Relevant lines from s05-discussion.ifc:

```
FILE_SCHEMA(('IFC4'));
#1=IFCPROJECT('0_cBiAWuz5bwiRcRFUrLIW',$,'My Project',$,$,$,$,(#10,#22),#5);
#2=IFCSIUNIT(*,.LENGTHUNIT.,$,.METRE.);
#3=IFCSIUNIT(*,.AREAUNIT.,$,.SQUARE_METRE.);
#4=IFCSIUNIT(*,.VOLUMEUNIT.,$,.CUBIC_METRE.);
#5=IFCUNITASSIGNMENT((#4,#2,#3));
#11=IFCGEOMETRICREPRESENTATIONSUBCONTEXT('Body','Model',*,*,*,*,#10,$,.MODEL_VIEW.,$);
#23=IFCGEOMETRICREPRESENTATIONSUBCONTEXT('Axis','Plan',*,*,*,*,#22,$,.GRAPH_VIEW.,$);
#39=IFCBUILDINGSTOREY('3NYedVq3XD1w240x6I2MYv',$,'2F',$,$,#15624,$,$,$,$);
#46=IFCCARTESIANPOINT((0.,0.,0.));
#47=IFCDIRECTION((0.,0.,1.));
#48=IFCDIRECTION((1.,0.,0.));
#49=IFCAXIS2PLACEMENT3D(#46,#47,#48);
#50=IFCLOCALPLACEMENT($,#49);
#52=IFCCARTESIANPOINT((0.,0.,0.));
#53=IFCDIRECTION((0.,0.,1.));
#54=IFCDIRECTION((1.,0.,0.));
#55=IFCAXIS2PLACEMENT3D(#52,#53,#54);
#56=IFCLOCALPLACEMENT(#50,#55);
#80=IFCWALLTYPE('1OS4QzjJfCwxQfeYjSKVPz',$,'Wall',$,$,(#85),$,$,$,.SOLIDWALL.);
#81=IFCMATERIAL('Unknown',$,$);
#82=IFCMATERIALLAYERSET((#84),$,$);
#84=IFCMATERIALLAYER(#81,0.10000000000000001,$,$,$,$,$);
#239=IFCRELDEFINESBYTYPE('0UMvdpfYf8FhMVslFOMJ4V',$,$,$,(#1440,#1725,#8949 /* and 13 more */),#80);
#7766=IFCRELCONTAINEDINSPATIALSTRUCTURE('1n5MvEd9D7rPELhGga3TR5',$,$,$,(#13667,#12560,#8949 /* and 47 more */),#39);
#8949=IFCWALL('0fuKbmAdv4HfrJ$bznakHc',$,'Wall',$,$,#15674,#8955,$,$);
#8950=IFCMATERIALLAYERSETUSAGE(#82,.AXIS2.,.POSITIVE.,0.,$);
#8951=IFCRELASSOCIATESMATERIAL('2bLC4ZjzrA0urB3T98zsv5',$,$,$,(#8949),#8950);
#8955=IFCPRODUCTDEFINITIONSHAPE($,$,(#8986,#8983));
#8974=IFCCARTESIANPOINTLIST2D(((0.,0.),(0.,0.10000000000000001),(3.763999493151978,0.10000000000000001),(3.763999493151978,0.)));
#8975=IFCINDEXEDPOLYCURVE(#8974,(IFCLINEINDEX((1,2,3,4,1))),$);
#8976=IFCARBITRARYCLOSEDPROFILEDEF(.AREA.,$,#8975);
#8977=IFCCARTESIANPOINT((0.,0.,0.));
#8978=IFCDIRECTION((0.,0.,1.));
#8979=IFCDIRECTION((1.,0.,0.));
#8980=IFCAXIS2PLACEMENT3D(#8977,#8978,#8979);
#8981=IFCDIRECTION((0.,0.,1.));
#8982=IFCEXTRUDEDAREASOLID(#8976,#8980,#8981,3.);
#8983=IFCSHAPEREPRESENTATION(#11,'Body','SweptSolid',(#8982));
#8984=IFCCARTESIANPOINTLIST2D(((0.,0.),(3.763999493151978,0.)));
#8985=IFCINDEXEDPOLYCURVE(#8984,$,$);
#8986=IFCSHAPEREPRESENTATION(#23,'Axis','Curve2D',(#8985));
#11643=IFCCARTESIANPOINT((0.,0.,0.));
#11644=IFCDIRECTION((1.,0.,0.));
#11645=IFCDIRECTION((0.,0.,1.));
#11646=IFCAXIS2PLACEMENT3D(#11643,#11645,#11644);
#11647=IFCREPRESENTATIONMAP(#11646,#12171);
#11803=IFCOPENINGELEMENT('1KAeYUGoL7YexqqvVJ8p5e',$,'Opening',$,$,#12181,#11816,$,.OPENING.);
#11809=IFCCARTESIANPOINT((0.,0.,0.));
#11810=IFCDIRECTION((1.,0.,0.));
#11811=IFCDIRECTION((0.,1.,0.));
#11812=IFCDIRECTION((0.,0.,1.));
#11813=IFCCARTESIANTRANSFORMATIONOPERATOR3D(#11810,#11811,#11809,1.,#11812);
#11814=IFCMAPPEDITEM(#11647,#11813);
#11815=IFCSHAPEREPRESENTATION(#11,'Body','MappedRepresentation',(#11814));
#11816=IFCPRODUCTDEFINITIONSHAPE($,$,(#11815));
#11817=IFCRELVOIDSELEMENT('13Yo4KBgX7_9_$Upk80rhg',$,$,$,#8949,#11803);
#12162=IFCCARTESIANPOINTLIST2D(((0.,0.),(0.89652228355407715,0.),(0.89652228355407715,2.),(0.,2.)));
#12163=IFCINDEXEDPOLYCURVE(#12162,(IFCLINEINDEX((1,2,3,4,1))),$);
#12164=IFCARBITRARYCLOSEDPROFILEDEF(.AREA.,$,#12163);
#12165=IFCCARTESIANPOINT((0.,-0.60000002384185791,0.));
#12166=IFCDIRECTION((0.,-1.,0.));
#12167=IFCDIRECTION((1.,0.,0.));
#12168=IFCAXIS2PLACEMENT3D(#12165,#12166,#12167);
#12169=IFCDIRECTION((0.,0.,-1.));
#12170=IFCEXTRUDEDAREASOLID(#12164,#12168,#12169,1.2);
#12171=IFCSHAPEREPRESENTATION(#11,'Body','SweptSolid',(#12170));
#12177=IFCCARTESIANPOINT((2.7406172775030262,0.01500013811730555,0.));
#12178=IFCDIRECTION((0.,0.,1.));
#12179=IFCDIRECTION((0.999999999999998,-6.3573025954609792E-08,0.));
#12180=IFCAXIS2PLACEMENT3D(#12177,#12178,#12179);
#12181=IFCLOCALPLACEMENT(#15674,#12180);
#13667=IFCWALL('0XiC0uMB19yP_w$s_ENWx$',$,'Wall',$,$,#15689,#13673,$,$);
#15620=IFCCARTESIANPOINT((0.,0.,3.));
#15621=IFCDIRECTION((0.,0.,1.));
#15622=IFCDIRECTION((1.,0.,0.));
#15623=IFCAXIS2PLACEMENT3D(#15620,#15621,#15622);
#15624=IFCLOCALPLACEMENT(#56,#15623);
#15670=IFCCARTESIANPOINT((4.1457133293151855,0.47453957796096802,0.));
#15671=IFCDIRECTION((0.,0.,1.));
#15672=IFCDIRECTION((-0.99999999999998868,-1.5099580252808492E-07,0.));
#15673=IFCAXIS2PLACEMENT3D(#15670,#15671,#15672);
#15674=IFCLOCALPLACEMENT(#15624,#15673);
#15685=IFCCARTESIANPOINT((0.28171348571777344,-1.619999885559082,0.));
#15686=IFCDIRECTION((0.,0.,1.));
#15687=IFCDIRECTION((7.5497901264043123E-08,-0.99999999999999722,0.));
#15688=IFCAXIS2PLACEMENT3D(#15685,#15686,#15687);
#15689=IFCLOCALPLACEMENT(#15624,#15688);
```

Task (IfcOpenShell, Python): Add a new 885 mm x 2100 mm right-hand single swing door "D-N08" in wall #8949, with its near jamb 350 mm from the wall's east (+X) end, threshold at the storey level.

```python
import numpy as np
import ifcopenshell
import ifcopenshell.api.feature
import ifcopenshell.api.geometry
import ifcopenshell.api.root
import ifcopenshell.api.spatial
import ifcopenshell.geom
import ifcopenshell.util.element
import ifcopenshell.util.placement
import ifcopenshell.util.representation
import ifcopenshell.util.shape
import ifcopenshell.util.unit

model = ifcopenshell.open("s05-discussion.ifc")
unit_scale = ifcopenshell.util.unit.calculate_unit_scale(model)
settings = ifcopenshell.geom.settings()


def volume(element):
    """Net volume in cubic metres, openings subtracted."""
    shape = ifcopenshell.geom.create_shape(settings, element)
    return ifcopenshell.util.shape.get_volume(shape.geometry)


wall = model.by_guid("0fuKbmAdv4HfrJ$bznakHc")
storey = ifcopenshell.util.element.get_container(wall, ifc_class="IfcBuildingStorey")
context = ifcopenshell.util.representation.get_context(model, "Model", "Body", "MODEL_VIEW")
before = volume(wall)

width, height, from_end, sill = 0.885, 2.1, 0.35, 0.0  # metres

# The wall runs along its own X axis, and the end named is its -X end.
wall_shape = ifcopenshell.geom.create_shape(settings, wall)
x, y, z = ifcopenshell.util.shape.get_vertices(wall_shape.geometry).T
start = x.min() + from_end
face, thickness = float(y.min()), float(y.max() - y.min())
wall_matrix = ifcopenshell.util.placement.get_local_placement(wall.ObjectPlacement)
level = ifcopenshell.util.placement.get_local_placement(storey.ObjectPlacement)[2, 3]


def in_wall(x, y):
    """Placement at x, y metres in the wall's axes, at sill height."""
    matrix = wall_matrix.copy()
    matrix[:, 3] = wall_matrix @ np.array([x / unit_scale, y / unit_scale, 0.0, 1.0])
    matrix[2, 3] = level + sill / unit_scale
    return matrix


# Opening: a box that overshoots both wall faces by 50 mm.
opening = ifcopenshell.api.root.create_entity(model, ifc_class="IfcOpeningElement", predefined_type="OPENING")
box = ifcopenshell.api.geometry.add_wall_representation(
    model, context=context, length=width, height=height, thickness=thickness + 0.1
)
ifcopenshell.api.geometry.assign_representation(model, product=opening, representation=box)
ifcopenshell.api.geometry.edit_object_placement(model, product=opening, matrix=in_wall(start, face - 0.05), is_si=False)
ifcopenshell.api.feature.add_feature(model, feature=opening, element=wall)

door = ifcopenshell.api.root.create_entity(model, ifc_class="IfcDoor", name="D-N08", predefined_type="DOOR")
door.OverallWidth, door.OverallHeight = width / unit_scale, height / unit_scale
door.OperationType = "SINGLE_SWING_RIGHT"
body = ifcopenshell.api.geometry.add_door_representation(
    model,
    context=context,
    overall_width=door.OverallWidth,
    overall_height=door.OverallHeight,
    operation_type="SINGLE_SWING_RIGHT",
    lining_properties={"LiningDepth": thickness / unit_scale, "ThresholdDepth": thickness / unit_scale},
)
ifcopenshell.api.geometry.assign_representation(model, product=door, representation=body)
ifcopenshell.api.spatial.assign_container(model, products=[door], relating_structure=storey)
ifcopenshell.api.feature.add_filling(model, opening=opening, element=door)

# The lining spans the wall, so the door starts at the wall face.
ifcopenshell.api.geometry.edit_object_placement(model, product=door, matrix=in_wall(start, face), is_si=False)

after = volume(wall)

print(f"wall volume {before:.3f} -> {after:.3f} m3")

model.write("s05-discussion_rev.ifc")
```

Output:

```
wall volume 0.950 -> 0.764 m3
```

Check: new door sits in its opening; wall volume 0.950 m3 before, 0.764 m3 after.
